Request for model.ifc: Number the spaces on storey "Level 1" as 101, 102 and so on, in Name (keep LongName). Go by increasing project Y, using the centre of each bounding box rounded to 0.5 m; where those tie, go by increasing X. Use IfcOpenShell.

First a look at what the model holds.

```python
import ifcopenshell
import ifcopenshell.util.element
import ifcopenshell.util.placement

model = ifcopenshell.open("model.ifc")
print(model.schema)
storey = next(s for s in model.by_type("IfcBuildingStorey") if s.Name == "Level 1")
spaces = [e for e in ifcopenshell.util.element.get_decomposition(storey) if e.is_a("IfcSpace")]
for e in sorted(spaces, key=lambda e: e.id()):
    origin = ifcopenshell.util.placement.get_local_placement(e.ObjectPlacement)[:3, 3]
    print(e.id(), e.Name, e.LongName, origin.round(2) + 0.0, sep=" | ")
```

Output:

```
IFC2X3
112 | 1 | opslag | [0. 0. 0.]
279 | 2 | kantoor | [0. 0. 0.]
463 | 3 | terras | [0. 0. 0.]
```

```python
import ifcopenshell
import ifcopenshell.geom
import ifcopenshell.util.element
import ifcopenshell.util.shape

model = ifcopenshell.open("model.ifc")
settings = ifcopenshell.geom.settings()
settings.set("use-world-coords", True)


def centre(element):
    shape = ifcopenshell.geom.create_shape(settings, element)
    return ifcopenshell.util.shape.get_bbox_centroid(shape.geometry)


storey = next(s for s in model.by_type("IfcBuildingStorey") if s.Name == "Level 1")
spaces = [e for e in ifcopenshell.util.element.get_decomposition(storey) if e.is_a("IfcSpace")]

# Insertion points can sit at a corner or the storey origin, so sort by the geometry (in metres).
centres = {e: centre(e) for e in spaces}
spaces.sort(key=lambda e: (round(centres[e][1] / 0.5), centres[e][0]))

for i, e in enumerate(spaces, start=1):
    number = f"1{i:02d}"
    e.Name = number
    print(e.id(), number)

model.write("model_edited.ifc")
```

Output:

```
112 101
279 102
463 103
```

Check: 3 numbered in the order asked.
